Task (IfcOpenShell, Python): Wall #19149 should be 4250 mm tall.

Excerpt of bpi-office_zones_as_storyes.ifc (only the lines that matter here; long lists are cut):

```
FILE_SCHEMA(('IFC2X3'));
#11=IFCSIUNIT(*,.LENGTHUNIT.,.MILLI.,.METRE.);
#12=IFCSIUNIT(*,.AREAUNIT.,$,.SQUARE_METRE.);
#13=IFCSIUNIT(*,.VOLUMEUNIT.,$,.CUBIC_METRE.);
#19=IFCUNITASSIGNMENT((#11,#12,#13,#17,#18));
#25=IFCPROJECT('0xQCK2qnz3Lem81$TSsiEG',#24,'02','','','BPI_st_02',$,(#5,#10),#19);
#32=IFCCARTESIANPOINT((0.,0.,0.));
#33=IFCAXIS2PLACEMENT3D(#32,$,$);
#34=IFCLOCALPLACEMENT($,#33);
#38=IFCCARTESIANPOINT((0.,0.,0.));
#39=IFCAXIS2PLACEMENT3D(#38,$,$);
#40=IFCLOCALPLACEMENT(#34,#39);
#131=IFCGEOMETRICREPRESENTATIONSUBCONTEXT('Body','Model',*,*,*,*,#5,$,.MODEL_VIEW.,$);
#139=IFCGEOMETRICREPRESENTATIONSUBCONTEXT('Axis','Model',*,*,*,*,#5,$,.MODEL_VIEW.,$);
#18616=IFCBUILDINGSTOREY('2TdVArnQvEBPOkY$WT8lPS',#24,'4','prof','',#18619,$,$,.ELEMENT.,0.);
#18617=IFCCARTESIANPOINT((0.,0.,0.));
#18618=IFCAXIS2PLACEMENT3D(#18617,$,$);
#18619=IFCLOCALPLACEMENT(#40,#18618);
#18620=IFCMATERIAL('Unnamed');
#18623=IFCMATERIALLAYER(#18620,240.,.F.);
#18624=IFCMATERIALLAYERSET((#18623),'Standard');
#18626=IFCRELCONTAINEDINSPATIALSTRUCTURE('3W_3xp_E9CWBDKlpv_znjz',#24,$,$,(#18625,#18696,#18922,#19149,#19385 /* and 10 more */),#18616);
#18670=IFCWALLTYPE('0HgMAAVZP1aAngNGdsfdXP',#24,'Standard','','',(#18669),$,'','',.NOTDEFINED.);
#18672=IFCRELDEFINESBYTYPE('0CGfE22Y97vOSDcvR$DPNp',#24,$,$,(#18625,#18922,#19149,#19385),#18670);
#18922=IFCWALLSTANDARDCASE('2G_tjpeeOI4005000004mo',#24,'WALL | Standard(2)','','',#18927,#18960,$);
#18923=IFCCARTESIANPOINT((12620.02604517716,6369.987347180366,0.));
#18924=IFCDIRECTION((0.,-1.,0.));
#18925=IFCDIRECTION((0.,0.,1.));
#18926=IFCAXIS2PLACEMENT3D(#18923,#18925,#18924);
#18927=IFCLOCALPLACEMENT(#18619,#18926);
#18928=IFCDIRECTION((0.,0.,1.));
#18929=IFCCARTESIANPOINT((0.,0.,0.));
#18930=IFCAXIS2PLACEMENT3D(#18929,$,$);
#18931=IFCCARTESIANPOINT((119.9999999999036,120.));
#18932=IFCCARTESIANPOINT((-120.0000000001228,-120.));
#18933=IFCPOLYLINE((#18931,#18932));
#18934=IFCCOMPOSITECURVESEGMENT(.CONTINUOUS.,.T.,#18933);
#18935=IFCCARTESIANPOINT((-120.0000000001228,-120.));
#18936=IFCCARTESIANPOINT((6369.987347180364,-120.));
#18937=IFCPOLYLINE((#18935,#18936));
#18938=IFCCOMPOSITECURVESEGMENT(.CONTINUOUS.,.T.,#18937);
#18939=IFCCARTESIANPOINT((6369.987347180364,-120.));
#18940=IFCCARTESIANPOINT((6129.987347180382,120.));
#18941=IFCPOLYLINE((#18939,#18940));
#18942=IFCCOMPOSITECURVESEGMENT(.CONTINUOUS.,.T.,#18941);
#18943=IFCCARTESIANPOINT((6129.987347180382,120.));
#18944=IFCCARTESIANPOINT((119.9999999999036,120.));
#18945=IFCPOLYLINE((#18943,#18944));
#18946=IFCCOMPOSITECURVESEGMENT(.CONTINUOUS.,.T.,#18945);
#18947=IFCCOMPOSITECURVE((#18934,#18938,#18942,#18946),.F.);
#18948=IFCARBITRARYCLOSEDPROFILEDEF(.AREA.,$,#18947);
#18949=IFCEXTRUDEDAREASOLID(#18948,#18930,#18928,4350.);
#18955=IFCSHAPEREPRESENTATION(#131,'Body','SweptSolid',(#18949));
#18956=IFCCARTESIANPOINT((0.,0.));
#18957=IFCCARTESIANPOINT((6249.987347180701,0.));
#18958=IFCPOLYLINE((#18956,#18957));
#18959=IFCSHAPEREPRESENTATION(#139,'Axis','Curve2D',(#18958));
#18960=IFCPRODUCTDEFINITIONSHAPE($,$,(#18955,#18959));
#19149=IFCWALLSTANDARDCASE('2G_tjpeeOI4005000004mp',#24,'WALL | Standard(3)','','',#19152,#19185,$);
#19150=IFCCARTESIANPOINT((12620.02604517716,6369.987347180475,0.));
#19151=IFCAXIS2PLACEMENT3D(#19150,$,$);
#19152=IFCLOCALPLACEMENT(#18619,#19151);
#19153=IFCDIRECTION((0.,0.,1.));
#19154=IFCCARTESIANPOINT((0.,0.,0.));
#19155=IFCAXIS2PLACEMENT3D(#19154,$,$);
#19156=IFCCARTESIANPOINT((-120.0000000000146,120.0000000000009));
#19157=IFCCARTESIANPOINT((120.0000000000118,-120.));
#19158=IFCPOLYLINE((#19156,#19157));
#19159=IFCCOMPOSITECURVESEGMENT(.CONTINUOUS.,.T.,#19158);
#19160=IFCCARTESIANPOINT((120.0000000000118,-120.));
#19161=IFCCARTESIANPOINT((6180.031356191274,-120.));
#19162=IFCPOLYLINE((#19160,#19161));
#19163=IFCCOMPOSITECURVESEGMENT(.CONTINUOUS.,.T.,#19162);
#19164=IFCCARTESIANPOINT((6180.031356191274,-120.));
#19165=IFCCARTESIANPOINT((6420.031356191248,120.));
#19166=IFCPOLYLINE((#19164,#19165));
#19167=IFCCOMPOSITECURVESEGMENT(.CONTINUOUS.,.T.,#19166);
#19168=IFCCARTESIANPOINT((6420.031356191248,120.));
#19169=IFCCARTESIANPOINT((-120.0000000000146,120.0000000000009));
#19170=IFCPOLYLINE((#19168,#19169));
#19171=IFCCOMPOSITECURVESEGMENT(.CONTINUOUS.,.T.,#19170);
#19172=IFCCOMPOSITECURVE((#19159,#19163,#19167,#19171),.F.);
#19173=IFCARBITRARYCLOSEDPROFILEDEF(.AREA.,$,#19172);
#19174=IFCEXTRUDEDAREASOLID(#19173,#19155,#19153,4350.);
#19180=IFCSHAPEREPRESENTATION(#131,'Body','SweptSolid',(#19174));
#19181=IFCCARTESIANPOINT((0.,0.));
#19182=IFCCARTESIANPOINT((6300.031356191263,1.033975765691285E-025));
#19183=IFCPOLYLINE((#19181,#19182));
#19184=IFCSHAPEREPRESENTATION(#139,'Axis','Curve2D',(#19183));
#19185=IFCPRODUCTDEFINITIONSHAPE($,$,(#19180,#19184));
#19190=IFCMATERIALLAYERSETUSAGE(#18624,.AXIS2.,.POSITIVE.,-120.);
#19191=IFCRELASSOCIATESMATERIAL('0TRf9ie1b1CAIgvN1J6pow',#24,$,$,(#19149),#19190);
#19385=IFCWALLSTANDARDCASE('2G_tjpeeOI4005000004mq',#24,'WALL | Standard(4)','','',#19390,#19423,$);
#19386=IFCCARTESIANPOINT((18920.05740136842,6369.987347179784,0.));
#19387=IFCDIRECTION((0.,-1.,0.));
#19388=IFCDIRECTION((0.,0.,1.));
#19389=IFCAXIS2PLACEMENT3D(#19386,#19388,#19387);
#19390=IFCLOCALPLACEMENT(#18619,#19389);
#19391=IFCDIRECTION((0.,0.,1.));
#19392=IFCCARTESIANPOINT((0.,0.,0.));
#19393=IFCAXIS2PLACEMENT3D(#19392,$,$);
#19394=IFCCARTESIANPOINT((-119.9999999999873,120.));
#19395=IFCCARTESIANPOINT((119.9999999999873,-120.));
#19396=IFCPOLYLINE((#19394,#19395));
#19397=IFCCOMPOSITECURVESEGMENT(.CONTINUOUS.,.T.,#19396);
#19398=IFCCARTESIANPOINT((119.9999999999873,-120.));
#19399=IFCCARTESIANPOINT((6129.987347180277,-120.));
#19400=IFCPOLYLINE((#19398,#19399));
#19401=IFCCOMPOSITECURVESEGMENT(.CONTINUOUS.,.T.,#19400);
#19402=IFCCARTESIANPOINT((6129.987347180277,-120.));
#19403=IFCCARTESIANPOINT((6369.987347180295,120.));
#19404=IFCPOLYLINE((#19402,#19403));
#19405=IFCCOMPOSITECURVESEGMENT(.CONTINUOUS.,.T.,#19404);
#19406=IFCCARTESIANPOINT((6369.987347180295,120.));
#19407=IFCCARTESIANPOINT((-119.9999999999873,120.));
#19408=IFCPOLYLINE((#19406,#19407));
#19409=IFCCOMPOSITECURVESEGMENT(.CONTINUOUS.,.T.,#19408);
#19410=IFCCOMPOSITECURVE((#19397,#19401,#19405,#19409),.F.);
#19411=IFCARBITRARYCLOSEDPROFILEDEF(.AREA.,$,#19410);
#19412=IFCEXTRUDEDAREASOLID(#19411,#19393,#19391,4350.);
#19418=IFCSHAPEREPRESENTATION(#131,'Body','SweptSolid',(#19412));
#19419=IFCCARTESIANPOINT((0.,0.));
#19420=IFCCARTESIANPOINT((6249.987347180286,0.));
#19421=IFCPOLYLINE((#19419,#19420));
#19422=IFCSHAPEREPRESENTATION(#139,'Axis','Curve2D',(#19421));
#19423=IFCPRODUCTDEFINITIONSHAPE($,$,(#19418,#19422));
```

```python
import ifcopenshell
import ifcopenshell.geom
import ifcopenshell.util.representation
import ifcopenshell.util.shape
import ifcopenshell.util.unit

model = ifcopenshell.open("bpi-office_zones_as_storyes.ifc")
unit_scale = ifcopenshell.util.unit.calculate_unit_scale(model)
settings = ifcopenshell.geom.settings()


def volume(element):
    """Net volume in cubic metres, openings subtracted."""
    shape = ifcopenshell.geom.create_shape(settings, element)
    return ifcopenshell.util.shape.get_volume(shape.geometry)


wall = model.by_guid("2G_tjpeeOI4005000004mp")
before = volume(wall)

body = ifcopenshell.util.representation.get_representation(wall, "Model", "Body")
solid = body.Items[0]
old_height = solid.Depth
solid.Depth = 4.25 / unit_scale
after = volume(wall)

print(f"height {old_height:g} -> {solid.Depth:g}, volume {before:.3f} -> {after:.3f} m3")

model.write("bpi-office_zones_as_storyes_edited.ifc")
```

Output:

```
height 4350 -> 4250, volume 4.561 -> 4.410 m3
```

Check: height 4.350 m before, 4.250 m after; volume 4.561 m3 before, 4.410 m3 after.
